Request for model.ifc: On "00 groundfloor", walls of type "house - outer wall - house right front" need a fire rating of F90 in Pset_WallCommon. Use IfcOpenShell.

First a look at what the model holds.

```python
import ifcopenshell
import ifcopenshell.util.element

model = ifcopenshell.open("model.ifc")
print(model.schema)
storey = next(s for s in model.by_type("IfcBuildingStorey") if s.Name == "00 groundfloor")
walls = [e for e in ifcopenshell.util.element.get_decomposition(storey) if e.is_a("IfcWall")]
seen = {}
for e in walls:
    element_type = ifcopenshell.util.element.get_type(e)
    key = (element_type.Name if element_type != e and element_type else None, ifcopenshell.util.element.get_pset(e, "Pset_WallCommon", "FireRating"))
    seen[key] = seen.get(key, 0) + 1
for (name, value), count in sorted(seen.items(), key=str):
    print(count, "x", name, "|", value)
```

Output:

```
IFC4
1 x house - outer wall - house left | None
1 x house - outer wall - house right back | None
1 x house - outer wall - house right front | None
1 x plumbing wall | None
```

```python
import ifcopenshell
import ifcopenshell.api.pset
import ifcopenshell.util.element

model = ifcopenshell.open("model.ifc")

storey = next(s for s in model.by_type("IfcBuildingStorey") if s.Name == "00 groundfloor")
walls = [e for e in ifcopenshell.util.element.get_decomposition(storey) if e.is_a("IfcWall")]

count = 0
for e in walls:
    element_type = ifcopenshell.util.element.get_type(e)
    if element_type in (None, e) or element_type.Name != "house - outer wall - house right front":
        continue
    # add_pset returns the element's existing set when there is one.
    pset = ifcopenshell.api.pset.add_pset(model, product=e, name="Pset_WallCommon")
    ifcopenshell.api.pset.edit_pset(model, pset=pset, properties={"FireRating": "F90"})
    count += 1

print(count, "walls updated")

model.write("model_edited.ifc")
```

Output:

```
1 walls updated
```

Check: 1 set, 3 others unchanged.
